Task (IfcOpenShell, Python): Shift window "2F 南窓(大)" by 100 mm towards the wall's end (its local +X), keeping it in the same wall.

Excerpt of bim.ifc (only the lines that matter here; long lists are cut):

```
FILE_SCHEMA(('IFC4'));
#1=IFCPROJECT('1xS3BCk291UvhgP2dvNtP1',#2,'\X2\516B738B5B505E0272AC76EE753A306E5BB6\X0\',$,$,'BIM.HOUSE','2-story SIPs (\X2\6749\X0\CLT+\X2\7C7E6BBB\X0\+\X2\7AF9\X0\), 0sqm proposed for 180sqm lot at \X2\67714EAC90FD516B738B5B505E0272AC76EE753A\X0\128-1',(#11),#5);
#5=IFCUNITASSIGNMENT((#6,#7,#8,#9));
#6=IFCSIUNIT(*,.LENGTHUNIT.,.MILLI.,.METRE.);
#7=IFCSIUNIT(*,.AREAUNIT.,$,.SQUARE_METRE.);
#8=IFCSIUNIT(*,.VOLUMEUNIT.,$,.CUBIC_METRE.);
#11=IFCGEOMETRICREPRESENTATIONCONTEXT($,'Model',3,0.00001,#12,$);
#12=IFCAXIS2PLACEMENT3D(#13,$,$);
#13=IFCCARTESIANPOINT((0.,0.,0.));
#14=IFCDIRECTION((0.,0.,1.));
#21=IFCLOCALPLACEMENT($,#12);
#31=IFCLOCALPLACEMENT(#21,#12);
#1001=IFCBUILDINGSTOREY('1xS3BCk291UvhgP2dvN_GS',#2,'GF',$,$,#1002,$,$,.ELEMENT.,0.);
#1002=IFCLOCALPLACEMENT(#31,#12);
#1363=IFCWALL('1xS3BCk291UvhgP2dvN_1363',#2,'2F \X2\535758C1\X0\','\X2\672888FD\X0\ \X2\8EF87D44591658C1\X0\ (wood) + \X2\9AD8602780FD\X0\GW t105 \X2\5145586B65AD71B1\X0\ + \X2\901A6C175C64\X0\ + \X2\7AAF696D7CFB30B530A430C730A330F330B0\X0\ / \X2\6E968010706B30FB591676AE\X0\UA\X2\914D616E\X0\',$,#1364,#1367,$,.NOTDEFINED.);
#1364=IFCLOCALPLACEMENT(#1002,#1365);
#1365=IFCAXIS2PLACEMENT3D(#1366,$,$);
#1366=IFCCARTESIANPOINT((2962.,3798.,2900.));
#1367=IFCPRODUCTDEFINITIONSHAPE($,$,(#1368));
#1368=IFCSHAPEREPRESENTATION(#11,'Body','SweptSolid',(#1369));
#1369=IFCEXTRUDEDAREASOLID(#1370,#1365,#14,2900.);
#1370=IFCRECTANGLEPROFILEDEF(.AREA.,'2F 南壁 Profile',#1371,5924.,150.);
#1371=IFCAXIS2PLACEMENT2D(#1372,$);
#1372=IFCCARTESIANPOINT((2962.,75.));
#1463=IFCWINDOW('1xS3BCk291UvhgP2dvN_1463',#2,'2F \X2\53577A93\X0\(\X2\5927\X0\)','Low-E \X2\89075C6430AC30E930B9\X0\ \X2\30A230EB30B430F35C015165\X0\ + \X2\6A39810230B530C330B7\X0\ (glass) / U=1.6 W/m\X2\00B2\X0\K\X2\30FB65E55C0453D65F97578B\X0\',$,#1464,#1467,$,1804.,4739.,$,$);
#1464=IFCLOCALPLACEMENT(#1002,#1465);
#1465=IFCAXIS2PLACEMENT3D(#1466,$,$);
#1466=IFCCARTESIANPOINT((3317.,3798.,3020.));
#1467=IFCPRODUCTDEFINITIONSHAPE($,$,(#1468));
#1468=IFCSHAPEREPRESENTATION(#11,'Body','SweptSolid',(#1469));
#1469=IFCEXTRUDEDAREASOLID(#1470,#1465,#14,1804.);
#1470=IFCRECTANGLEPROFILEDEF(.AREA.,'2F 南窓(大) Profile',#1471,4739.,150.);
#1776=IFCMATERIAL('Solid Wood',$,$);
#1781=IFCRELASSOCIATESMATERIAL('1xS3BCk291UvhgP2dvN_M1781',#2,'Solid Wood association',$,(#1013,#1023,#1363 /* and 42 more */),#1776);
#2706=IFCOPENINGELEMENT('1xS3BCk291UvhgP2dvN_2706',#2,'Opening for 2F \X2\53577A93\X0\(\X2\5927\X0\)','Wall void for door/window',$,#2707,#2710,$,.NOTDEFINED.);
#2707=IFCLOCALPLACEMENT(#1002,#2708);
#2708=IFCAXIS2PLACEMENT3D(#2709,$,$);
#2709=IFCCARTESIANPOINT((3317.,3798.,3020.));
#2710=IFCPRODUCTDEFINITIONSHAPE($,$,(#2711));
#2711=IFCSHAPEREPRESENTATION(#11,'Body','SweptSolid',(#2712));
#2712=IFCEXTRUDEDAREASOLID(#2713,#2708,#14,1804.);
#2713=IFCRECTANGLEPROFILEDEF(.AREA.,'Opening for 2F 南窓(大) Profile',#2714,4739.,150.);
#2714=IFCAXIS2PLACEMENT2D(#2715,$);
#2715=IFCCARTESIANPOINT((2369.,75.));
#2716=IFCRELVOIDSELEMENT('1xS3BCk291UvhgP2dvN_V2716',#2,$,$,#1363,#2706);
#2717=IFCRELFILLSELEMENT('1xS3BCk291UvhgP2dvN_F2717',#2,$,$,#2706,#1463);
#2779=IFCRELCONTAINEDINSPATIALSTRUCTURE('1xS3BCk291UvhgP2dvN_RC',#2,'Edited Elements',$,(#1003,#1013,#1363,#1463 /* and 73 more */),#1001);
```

```python
import ifcopenshell
import ifcopenshell.api.geometry
import ifcopenshell.util.placement
import ifcopenshell.util.unit

model = ifcopenshell.open("bim.ifc")
unit_scale = ifcopenshell.util.unit.calculate_unit_scale(model)

window = model.by_guid("1xS3BCk291UvhgP2dvN_1463")
opening = window.FillsVoids[0].RelatingOpeningElement
wall = opening.VoidsElements[0].RelatingBuildingElement

wall_matrix = ifcopenshell.util.placement.get_local_placement(wall.ObjectPlacement)
shift = wall_matrix[:3, 0] * 0.1 / unit_scale
before = ifcopenshell.util.placement.get_local_placement(window.ObjectPlacement)[:3, 3].copy()

# The window is not placed relative to its opening, so move both.
for product in (opening, window):
    matrix = ifcopenshell.util.placement.get_local_placement(product.ObjectPlacement)
    matrix[:3, 3] += shift
    ifcopenshell.api.geometry.edit_object_placement(model, product=product, matrix=matrix, is_si=False)

after = ifcopenshell.util.placement.get_local_placement(window.ObjectPlacement)[:3, 3]
print("window moved by", (after - before).round(3) + 0.0)

model.write("bim_v2.ifc")
```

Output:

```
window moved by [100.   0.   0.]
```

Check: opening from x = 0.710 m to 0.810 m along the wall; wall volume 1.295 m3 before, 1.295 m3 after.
